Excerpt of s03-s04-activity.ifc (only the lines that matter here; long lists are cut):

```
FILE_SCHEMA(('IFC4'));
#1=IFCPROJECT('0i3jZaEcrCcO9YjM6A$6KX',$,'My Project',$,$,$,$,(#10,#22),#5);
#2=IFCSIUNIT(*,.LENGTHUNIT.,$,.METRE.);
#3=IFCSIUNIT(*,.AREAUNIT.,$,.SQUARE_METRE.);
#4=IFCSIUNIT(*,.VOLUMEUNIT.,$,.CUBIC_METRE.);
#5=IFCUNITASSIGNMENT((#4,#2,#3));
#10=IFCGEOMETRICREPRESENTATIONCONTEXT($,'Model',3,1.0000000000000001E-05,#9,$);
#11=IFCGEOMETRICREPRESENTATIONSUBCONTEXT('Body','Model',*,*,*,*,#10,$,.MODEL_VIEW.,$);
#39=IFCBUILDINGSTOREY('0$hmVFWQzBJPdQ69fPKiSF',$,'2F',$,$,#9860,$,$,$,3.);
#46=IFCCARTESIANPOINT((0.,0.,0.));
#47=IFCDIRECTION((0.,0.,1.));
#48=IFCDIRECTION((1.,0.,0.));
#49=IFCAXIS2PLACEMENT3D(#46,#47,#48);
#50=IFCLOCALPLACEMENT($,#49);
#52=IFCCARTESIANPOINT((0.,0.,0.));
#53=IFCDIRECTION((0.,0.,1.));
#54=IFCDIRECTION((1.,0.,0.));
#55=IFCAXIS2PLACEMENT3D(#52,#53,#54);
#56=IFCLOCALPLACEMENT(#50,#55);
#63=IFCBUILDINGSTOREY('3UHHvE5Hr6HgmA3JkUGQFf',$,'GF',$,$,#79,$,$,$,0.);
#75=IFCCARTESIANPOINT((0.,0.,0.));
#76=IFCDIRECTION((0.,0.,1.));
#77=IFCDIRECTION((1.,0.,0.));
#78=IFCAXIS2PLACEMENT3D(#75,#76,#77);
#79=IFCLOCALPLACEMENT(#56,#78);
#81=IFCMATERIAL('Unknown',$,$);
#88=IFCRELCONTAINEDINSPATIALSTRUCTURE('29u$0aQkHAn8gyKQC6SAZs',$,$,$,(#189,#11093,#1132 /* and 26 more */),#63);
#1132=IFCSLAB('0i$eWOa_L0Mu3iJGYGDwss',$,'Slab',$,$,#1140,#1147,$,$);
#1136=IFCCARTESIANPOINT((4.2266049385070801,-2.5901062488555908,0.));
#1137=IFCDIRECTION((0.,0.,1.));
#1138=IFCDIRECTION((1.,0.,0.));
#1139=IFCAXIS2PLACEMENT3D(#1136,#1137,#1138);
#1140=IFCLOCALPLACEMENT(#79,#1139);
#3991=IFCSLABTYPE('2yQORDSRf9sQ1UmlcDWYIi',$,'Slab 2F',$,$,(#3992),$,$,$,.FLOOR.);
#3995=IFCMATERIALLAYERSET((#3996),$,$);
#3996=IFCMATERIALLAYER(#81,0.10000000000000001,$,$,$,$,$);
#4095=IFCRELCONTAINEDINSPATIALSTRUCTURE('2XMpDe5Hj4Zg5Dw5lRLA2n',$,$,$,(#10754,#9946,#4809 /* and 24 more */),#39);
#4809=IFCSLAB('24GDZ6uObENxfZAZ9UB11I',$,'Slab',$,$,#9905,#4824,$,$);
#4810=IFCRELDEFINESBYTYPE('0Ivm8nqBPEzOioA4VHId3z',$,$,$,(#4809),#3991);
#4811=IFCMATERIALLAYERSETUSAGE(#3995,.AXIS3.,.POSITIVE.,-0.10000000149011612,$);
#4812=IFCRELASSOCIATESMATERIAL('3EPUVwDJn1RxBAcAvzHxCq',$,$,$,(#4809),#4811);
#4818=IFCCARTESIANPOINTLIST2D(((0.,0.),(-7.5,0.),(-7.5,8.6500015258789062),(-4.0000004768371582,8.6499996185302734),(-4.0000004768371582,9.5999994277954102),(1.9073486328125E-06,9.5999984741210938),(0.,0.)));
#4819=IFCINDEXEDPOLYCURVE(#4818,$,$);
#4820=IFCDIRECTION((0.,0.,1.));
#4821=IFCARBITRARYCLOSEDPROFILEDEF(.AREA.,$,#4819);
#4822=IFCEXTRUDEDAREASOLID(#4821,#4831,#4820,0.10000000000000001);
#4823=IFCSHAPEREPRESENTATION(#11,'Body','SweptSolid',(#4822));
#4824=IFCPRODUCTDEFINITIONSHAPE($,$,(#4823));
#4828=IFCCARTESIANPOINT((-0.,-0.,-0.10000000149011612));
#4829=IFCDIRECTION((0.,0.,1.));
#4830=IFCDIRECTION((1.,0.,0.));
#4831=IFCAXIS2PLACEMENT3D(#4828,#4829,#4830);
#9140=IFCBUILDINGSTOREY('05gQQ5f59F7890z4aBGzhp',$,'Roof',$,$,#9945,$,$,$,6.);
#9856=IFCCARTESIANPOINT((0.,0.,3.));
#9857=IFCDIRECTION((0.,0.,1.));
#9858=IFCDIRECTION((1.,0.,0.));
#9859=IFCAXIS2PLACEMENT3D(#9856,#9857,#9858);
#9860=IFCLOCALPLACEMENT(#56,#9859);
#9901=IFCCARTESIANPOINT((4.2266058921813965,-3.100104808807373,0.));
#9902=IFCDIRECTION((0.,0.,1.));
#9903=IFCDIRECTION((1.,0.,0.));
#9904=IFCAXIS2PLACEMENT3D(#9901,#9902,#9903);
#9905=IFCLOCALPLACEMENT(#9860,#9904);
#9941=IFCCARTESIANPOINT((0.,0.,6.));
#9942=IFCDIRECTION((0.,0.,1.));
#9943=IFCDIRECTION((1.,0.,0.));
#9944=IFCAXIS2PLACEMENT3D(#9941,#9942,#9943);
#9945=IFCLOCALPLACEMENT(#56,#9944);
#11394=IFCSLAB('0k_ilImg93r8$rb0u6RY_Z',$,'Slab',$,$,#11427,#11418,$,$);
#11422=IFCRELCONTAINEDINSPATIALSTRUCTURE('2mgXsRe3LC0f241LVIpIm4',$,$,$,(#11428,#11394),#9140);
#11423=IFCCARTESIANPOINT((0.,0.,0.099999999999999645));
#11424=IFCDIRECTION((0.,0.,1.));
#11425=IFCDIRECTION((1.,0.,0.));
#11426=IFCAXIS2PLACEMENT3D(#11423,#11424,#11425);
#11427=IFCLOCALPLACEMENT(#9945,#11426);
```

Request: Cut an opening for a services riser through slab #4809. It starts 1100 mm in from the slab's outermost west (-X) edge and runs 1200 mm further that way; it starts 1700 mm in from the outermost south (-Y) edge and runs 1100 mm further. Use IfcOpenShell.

```python
import numpy as np
import ifcopenshell
import ifcopenshell.api.feature
import ifcopenshell.api.geometry
import ifcopenshell.api.root
import ifcopenshell.geom
import ifcopenshell.util.placement
import ifcopenshell.util.representation
import ifcopenshell.util.shape
import ifcopenshell.util.unit

model = ifcopenshell.open("s03-s04-activity.ifc")
unit_scale = ifcopenshell.util.unit.calculate_unit_scale(model)
settings = ifcopenshell.geom.settings()


def volume(element):
    """Net volume in cubic metres, openings subtracted."""
    shape = ifcopenshell.geom.create_shape(settings, element)
    return ifcopenshell.util.shape.get_volume(shape.geometry)


slab = model.by_id(4809)
before = volume(slab)

# Extent in the slab's own axes, in metres. The edges named are its -X and -Y sides.
slab_shape = ifcopenshell.geom.create_shape(settings, slab)
vertices = ifcopenshell.util.shape.get_vertices(slab_shape.geometry)
x_min, y_min, bottom = vertices.min(axis=0)
top = vertices[:, 2].max()

opening = ifcopenshell.api.root.create_entity(model, ifc_class="IfcOpeningElement", name="Services riser opening", predefined_type="OPENING")
context = ifcopenshell.util.representation.get_context(model, "Model", "Body", "MODEL_VIEW")
width, depth = 1.2, 1.1
outline = [(0.0, 0.0), (width, 0.0), (width, depth), (0.0, depth), (0.0, 0.0)]
# Overshoot both faces by 50 mm so the cut is clean.
shape = ifcopenshell.api.geometry.add_slab_representation(
    model, context=context, depth=top - bottom + 0.1, polyline=outline
)
ifcopenshell.api.geometry.assign_representation(model, product=opening, representation=shape)

matrix = ifcopenshell.util.placement.get_local_placement(slab.ObjectPlacement)
matrix[:, 3] = matrix @ np.append(np.array([x_min + 1.1, y_min + 1.7, bottom - 0.05]) / unit_scale, 1.0)
ifcopenshell.api.geometry.edit_object_placement(model, product=opening, matrix=matrix, is_si=False)
ifcopenshell.api.feature.add_feature(model, feature=opening, element=slab)

after = volume(slab)

print(f"slab volume {before:.3f} -> {after:.3f} m3")

model.write("s03-s04-activity-out.ifc")
```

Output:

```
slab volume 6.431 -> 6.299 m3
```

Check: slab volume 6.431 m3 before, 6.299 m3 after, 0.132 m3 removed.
